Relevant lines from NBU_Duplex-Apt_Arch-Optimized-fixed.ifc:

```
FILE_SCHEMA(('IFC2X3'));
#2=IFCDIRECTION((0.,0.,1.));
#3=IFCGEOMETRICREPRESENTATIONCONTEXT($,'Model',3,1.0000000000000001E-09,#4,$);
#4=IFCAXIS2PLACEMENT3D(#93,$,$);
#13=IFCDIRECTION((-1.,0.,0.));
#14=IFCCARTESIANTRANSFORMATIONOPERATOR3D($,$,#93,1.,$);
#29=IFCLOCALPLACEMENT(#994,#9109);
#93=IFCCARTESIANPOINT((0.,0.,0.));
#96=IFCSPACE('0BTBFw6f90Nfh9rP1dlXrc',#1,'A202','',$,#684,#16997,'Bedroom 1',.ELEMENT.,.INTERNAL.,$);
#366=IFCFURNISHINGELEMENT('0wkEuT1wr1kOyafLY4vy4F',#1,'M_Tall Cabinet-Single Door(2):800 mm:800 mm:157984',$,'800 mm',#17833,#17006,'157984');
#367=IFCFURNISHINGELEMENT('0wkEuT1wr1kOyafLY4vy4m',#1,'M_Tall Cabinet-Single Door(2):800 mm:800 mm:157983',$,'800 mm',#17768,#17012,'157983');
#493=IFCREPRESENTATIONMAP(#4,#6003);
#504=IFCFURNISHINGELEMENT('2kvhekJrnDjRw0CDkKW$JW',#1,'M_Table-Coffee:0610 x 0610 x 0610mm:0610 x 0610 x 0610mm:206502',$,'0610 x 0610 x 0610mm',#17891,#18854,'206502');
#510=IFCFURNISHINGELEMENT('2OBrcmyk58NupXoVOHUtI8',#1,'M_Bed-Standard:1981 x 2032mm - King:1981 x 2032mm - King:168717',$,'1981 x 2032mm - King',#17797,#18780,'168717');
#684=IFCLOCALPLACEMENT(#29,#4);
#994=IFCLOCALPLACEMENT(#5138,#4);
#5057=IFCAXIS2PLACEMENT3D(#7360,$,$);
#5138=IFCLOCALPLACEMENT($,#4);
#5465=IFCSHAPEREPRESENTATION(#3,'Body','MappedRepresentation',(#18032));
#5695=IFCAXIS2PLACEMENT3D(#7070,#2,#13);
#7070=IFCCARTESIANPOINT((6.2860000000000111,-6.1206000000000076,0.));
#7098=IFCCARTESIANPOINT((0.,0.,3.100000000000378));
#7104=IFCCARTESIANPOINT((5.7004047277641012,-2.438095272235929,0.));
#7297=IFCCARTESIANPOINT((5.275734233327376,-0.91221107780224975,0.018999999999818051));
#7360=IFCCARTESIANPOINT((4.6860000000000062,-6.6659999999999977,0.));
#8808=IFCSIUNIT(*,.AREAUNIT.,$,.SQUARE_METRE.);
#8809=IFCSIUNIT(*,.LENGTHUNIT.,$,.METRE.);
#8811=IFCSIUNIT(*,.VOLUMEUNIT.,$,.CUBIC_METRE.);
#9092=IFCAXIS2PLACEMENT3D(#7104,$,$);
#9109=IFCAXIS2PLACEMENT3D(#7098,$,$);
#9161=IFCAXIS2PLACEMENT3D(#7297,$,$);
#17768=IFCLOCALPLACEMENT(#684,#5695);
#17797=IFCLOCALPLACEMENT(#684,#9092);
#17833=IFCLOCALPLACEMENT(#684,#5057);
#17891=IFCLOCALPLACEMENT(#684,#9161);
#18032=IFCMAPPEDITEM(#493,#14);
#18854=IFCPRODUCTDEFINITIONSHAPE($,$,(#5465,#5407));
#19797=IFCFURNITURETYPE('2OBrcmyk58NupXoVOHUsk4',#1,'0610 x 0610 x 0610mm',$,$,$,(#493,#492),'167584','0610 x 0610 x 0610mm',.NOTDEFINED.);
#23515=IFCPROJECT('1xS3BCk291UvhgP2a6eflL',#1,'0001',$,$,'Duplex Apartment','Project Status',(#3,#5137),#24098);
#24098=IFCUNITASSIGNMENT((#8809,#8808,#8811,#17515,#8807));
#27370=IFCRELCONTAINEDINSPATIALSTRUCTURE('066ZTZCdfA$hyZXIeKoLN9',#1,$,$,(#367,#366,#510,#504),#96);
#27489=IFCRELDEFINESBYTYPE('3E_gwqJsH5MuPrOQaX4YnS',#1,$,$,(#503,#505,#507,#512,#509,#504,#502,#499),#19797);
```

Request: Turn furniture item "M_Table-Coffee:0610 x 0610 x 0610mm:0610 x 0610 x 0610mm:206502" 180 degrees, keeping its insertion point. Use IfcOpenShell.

```python
import ifcopenshell
import ifcopenshell.api.geometry
import ifcopenshell.util.placement

model = ifcopenshell.open("NBU_Duplex-Apt_Arch-Optimized-fixed.ifc")

item = model.by_guid("2kvhekJrnDjRw0CDkKW$JW")
matrix = ifcopenshell.util.placement.get_local_placement(item.ObjectPlacement)
matrix = matrix @ ifcopenshell.util.placement.rotation(180, "Z")
ifcopenshell.api.geometry.edit_object_placement(model, product=item, matrix=matrix, is_si=False)

print(ifcopenshell.util.placement.get_local_placement(item.ObjectPlacement).round(3) + 0.0)

model.write("NBU_Duplex-Apt_Arch-Optimized-fixed_v2.ifc")
```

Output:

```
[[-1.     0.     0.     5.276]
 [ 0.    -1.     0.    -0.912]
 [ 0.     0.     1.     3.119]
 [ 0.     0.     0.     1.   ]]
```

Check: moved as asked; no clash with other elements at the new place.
